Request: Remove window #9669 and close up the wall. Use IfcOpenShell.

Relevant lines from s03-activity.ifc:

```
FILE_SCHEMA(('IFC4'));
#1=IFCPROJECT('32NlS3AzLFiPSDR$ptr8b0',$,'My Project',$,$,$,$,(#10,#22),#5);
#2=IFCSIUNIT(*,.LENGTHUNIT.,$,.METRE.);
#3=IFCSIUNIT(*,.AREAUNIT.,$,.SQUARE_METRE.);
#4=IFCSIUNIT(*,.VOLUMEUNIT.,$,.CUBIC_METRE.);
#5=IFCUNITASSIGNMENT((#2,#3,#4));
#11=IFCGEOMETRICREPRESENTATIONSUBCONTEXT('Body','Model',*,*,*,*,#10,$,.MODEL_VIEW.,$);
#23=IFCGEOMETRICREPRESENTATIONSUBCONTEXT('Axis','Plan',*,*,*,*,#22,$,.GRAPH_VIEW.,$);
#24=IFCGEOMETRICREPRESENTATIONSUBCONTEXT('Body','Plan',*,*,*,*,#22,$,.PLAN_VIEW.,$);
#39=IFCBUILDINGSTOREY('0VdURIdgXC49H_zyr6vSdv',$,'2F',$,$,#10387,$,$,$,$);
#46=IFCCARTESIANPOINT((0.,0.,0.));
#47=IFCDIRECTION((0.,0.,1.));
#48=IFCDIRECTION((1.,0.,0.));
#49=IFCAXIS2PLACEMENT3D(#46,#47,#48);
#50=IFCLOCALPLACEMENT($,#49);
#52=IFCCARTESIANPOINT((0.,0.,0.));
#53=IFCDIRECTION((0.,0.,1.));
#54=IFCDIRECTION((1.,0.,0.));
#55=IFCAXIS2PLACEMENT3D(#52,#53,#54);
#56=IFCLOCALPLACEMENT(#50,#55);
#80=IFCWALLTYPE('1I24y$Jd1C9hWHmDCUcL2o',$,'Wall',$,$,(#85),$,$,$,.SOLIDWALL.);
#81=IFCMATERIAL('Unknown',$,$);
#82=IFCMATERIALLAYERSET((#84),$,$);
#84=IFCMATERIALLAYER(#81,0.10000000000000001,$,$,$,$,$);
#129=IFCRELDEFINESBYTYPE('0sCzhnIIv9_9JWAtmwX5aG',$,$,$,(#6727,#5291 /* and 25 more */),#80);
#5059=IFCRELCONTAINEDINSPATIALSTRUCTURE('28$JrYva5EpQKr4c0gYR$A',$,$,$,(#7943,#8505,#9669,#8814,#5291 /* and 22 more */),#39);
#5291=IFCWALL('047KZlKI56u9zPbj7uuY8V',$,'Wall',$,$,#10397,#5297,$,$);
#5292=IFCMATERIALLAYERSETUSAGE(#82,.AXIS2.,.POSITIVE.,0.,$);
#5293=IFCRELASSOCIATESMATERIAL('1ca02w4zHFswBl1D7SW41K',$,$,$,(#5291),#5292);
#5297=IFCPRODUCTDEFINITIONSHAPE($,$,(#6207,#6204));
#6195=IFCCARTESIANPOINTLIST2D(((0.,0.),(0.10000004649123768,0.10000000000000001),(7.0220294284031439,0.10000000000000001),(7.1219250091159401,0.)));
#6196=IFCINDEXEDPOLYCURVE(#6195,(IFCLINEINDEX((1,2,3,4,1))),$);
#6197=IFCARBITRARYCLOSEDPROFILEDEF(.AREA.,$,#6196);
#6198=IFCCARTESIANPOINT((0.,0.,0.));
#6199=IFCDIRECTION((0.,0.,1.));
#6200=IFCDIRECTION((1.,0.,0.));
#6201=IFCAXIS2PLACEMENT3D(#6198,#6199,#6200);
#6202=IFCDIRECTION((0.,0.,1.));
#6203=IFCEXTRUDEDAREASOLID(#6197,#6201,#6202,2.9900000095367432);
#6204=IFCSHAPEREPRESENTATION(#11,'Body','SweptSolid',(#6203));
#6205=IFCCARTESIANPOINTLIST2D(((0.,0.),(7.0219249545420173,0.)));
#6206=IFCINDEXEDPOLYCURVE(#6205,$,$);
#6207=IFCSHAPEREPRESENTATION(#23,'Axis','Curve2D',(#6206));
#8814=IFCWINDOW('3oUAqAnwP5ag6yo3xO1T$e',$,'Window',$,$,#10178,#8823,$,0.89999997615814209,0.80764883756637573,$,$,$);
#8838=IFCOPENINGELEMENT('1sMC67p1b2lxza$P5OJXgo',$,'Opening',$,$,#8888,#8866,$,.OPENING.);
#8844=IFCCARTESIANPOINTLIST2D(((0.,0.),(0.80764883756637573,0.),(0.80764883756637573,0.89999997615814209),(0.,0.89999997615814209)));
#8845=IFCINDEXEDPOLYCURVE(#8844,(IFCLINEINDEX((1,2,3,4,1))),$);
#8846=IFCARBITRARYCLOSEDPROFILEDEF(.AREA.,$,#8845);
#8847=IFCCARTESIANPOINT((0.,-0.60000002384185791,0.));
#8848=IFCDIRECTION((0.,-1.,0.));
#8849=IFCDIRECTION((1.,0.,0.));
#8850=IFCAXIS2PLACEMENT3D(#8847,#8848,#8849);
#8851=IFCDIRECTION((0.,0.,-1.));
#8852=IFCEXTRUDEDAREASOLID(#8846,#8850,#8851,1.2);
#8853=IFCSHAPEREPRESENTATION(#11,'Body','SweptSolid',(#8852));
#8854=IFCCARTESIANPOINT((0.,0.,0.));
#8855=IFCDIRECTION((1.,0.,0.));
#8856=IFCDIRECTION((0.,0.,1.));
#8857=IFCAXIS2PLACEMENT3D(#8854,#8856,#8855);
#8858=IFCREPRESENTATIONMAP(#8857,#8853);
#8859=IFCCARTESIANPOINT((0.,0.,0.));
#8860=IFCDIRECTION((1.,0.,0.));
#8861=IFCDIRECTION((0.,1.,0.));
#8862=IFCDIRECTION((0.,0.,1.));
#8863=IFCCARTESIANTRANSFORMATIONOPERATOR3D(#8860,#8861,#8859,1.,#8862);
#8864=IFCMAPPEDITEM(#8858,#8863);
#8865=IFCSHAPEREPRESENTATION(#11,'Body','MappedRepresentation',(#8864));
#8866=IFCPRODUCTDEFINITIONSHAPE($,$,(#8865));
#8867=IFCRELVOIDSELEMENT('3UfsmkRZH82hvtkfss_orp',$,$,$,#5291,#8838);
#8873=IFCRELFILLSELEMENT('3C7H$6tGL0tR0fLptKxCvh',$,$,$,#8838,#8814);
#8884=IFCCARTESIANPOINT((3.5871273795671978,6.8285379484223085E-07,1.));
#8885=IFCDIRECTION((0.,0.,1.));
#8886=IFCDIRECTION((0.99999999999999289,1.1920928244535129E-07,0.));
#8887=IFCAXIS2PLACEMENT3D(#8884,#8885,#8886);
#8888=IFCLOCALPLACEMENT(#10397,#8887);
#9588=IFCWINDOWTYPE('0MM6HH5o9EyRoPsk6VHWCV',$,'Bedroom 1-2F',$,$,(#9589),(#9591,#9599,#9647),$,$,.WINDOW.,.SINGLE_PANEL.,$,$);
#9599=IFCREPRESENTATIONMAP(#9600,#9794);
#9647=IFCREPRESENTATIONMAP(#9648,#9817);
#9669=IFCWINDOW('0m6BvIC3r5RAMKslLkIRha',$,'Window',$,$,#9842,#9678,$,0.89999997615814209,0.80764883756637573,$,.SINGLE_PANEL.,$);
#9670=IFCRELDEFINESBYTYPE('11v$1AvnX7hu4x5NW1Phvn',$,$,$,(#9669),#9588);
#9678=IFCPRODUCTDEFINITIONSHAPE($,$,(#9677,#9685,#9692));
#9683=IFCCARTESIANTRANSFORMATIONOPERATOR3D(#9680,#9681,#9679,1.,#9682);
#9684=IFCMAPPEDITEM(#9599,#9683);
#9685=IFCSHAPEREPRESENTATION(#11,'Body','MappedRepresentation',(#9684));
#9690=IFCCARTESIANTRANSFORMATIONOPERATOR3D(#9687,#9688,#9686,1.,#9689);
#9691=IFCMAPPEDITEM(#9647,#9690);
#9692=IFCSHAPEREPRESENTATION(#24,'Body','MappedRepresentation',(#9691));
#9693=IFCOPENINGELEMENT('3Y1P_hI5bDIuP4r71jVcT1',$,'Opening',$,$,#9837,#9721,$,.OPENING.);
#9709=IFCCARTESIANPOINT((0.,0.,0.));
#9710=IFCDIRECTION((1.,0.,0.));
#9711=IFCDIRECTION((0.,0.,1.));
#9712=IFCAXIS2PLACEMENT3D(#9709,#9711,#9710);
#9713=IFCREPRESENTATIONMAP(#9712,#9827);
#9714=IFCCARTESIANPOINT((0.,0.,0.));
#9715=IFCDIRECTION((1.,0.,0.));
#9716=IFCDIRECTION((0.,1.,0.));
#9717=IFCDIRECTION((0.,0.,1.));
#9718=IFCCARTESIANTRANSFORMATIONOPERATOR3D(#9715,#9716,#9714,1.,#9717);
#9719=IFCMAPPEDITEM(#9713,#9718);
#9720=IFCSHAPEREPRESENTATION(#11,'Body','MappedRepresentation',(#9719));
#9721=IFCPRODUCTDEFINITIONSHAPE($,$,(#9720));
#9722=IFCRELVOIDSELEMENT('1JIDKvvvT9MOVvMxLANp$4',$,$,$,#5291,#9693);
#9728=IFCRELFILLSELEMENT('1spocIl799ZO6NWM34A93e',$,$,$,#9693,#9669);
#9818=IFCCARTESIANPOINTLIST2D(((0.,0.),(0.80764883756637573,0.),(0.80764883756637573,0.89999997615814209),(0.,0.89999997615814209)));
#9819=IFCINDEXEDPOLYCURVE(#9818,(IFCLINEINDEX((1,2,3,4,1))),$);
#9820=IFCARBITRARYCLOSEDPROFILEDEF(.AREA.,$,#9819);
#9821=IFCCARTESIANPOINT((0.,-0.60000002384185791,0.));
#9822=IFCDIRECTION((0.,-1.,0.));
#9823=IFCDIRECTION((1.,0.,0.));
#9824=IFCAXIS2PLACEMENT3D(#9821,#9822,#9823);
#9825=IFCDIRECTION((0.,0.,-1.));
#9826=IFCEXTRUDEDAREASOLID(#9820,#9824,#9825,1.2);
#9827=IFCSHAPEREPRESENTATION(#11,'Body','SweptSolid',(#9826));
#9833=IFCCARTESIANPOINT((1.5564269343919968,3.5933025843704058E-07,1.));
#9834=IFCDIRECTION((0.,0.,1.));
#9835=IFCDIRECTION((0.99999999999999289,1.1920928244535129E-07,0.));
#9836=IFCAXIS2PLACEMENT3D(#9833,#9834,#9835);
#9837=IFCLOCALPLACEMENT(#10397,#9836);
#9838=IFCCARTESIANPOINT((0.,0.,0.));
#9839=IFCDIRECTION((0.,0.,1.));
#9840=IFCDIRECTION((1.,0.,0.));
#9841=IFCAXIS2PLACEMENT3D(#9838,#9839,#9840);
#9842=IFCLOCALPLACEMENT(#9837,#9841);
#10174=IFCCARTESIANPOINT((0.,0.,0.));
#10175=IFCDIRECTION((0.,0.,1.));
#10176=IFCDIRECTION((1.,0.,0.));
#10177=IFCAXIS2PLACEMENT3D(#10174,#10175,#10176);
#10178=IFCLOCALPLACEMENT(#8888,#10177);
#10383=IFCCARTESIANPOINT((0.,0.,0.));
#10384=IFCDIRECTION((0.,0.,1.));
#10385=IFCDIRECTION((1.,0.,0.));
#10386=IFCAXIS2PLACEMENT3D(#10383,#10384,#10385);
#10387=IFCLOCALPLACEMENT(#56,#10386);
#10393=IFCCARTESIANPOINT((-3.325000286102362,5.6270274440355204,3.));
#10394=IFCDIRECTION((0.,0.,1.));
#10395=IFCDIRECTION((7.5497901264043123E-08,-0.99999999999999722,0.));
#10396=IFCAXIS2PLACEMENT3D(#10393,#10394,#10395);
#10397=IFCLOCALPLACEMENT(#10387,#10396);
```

```python
import ifcopenshell
import ifcopenshell.api.feature
import ifcopenshell.api.root
import ifcopenshell.geom
import ifcopenshell.util.shape

model = ifcopenshell.open("s03-activity.ifc")
settings = ifcopenshell.geom.settings()


def volume(element):
    """Net volume in cubic metres, openings subtracted."""
    shape = ifcopenshell.geom.create_shape(settings, element)
    return ifcopenshell.util.shape.get_volume(shape.geometry)


window = model.by_guid("0m6BvIC3r5RAMKslLkIRha")
opening = window.FillsVoids[0].RelatingOpeningElement
wall = opening.VoidsElements[0].RelatingBuildingElement
before = volume(wall)

ifcopenshell.api.root.remove_product(model, product=window)
ifcopenshell.api.feature.remove_feature(model, feature=opening)

after = volume(wall)

print(f"wall volume {before:.3f} -> {after:.3f} m3")

model.write("s03-activity_rev.ifc")
```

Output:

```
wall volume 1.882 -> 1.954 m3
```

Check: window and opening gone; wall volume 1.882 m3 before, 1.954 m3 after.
